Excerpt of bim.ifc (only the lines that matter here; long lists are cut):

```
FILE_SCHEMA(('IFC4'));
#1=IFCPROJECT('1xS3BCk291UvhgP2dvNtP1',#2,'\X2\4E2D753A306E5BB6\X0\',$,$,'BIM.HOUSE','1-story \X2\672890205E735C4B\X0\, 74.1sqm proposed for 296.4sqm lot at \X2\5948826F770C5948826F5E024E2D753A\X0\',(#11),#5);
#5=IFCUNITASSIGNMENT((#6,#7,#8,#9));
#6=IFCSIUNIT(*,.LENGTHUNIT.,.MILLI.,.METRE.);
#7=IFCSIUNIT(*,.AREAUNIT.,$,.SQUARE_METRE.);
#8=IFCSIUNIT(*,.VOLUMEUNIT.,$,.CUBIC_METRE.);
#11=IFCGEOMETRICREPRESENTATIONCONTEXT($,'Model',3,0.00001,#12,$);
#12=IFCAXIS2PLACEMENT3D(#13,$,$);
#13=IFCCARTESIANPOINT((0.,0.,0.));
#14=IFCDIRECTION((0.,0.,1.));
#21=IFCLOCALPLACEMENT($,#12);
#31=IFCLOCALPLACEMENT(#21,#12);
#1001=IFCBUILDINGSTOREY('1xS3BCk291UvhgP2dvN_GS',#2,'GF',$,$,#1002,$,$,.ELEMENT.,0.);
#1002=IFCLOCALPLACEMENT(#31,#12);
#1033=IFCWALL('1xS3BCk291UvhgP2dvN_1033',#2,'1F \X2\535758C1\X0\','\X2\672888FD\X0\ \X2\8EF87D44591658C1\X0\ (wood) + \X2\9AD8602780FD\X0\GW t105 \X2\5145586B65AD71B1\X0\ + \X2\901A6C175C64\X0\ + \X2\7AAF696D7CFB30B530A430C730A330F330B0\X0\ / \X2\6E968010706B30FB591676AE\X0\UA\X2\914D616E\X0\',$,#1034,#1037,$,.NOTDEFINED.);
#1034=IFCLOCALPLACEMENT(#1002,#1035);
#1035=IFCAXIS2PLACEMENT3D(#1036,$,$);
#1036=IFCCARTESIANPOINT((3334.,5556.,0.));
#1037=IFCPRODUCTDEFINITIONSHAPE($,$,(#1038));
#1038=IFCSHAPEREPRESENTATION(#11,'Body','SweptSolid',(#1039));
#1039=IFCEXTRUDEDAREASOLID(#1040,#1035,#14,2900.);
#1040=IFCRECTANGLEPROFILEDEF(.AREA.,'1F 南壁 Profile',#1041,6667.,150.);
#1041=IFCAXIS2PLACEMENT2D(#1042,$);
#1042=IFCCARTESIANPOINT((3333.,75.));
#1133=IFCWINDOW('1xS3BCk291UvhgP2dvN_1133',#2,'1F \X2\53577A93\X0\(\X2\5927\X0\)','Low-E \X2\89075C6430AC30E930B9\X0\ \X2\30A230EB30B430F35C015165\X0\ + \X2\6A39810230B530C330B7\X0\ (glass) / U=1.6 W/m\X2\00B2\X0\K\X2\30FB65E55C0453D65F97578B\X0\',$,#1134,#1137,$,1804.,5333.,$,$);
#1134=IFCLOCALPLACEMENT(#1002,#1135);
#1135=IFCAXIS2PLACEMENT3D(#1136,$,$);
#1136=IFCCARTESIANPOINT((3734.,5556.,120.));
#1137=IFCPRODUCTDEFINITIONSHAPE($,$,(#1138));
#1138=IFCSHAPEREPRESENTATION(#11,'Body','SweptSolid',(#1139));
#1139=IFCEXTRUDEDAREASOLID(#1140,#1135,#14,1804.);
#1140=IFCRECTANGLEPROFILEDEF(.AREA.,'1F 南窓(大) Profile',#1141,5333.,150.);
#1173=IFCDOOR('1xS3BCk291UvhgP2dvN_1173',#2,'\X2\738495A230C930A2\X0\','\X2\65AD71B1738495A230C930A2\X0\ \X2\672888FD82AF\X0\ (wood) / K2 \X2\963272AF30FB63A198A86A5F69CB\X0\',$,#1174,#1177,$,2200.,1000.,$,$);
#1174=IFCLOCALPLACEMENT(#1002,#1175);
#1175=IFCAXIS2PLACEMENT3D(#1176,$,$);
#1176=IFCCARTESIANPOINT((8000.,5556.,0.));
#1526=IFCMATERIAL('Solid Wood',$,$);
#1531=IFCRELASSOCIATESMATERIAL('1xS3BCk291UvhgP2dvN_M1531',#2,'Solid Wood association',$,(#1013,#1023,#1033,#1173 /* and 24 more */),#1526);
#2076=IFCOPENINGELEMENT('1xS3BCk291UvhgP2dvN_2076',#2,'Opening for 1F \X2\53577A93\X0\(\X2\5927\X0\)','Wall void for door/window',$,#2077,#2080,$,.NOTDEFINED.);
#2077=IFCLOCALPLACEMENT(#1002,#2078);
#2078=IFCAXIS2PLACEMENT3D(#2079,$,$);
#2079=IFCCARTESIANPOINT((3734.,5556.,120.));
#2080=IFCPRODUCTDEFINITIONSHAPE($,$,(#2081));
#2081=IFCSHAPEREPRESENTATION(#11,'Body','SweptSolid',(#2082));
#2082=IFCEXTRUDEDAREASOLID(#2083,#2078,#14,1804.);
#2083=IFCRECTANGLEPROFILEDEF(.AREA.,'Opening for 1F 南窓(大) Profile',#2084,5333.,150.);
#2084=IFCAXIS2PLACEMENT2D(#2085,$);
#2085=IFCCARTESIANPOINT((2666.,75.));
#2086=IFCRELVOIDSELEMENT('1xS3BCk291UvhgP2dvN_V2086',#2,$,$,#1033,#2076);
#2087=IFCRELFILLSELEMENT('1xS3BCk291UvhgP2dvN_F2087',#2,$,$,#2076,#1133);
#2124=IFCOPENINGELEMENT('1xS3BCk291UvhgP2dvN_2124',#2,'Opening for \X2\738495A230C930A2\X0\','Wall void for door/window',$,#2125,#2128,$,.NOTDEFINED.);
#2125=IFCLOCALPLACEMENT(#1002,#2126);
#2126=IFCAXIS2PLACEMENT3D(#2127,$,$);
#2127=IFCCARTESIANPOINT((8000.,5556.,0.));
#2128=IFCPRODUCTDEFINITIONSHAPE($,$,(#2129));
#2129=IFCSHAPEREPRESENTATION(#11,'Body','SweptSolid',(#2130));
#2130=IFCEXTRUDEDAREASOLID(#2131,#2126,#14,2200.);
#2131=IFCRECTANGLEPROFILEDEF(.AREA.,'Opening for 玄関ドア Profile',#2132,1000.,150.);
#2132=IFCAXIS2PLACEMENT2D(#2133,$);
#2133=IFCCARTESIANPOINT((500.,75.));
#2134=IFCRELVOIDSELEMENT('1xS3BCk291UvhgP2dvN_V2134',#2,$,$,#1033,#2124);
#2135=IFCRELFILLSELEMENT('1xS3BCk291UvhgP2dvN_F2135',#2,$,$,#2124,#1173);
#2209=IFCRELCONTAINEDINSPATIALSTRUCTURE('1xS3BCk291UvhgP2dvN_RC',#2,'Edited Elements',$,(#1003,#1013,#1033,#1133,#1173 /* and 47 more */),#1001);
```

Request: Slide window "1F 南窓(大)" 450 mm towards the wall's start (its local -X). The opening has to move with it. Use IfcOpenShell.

```python
import ifcopenshell
import ifcopenshell.api.geometry
import ifcopenshell.util.placement
import ifcopenshell.util.unit

model = ifcopenshell.open("bim.ifc")
unit_scale = ifcopenshell.util.unit.calculate_unit_scale(model)

window = model.by_guid("1xS3BCk291UvhgP2dvN_1133")
opening = window.FillsVoids[0].RelatingOpeningElement
wall = opening.VoidsElements[0].RelatingBuildingElement

wall_matrix = ifcopenshell.util.placement.get_local_placement(wall.ObjectPlacement)
shift = wall_matrix[:3, 0] * -0.45 / unit_scale
before = ifcopenshell.util.placement.get_local_placement(window.ObjectPlacement)[:3, 3].copy()

# The window is not placed relative to its opening, so move both.
for product in (opening, window):
    matrix = ifcopenshell.util.placement.get_local_placement(product.ObjectPlacement)
    matrix[:3, 3] += shift
    ifcopenshell.api.geometry.edit_object_placement(model, product=product, matrix=matrix, is_si=False)

after = ifcopenshell.util.placement.get_local_placement(window.ObjectPlacement)[:3, 3]
print("window moved by", (after - before).round(3) + 0.0)

model.write("bim_rev.ifc")
```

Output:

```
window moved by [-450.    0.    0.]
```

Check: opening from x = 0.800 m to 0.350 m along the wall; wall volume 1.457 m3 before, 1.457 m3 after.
